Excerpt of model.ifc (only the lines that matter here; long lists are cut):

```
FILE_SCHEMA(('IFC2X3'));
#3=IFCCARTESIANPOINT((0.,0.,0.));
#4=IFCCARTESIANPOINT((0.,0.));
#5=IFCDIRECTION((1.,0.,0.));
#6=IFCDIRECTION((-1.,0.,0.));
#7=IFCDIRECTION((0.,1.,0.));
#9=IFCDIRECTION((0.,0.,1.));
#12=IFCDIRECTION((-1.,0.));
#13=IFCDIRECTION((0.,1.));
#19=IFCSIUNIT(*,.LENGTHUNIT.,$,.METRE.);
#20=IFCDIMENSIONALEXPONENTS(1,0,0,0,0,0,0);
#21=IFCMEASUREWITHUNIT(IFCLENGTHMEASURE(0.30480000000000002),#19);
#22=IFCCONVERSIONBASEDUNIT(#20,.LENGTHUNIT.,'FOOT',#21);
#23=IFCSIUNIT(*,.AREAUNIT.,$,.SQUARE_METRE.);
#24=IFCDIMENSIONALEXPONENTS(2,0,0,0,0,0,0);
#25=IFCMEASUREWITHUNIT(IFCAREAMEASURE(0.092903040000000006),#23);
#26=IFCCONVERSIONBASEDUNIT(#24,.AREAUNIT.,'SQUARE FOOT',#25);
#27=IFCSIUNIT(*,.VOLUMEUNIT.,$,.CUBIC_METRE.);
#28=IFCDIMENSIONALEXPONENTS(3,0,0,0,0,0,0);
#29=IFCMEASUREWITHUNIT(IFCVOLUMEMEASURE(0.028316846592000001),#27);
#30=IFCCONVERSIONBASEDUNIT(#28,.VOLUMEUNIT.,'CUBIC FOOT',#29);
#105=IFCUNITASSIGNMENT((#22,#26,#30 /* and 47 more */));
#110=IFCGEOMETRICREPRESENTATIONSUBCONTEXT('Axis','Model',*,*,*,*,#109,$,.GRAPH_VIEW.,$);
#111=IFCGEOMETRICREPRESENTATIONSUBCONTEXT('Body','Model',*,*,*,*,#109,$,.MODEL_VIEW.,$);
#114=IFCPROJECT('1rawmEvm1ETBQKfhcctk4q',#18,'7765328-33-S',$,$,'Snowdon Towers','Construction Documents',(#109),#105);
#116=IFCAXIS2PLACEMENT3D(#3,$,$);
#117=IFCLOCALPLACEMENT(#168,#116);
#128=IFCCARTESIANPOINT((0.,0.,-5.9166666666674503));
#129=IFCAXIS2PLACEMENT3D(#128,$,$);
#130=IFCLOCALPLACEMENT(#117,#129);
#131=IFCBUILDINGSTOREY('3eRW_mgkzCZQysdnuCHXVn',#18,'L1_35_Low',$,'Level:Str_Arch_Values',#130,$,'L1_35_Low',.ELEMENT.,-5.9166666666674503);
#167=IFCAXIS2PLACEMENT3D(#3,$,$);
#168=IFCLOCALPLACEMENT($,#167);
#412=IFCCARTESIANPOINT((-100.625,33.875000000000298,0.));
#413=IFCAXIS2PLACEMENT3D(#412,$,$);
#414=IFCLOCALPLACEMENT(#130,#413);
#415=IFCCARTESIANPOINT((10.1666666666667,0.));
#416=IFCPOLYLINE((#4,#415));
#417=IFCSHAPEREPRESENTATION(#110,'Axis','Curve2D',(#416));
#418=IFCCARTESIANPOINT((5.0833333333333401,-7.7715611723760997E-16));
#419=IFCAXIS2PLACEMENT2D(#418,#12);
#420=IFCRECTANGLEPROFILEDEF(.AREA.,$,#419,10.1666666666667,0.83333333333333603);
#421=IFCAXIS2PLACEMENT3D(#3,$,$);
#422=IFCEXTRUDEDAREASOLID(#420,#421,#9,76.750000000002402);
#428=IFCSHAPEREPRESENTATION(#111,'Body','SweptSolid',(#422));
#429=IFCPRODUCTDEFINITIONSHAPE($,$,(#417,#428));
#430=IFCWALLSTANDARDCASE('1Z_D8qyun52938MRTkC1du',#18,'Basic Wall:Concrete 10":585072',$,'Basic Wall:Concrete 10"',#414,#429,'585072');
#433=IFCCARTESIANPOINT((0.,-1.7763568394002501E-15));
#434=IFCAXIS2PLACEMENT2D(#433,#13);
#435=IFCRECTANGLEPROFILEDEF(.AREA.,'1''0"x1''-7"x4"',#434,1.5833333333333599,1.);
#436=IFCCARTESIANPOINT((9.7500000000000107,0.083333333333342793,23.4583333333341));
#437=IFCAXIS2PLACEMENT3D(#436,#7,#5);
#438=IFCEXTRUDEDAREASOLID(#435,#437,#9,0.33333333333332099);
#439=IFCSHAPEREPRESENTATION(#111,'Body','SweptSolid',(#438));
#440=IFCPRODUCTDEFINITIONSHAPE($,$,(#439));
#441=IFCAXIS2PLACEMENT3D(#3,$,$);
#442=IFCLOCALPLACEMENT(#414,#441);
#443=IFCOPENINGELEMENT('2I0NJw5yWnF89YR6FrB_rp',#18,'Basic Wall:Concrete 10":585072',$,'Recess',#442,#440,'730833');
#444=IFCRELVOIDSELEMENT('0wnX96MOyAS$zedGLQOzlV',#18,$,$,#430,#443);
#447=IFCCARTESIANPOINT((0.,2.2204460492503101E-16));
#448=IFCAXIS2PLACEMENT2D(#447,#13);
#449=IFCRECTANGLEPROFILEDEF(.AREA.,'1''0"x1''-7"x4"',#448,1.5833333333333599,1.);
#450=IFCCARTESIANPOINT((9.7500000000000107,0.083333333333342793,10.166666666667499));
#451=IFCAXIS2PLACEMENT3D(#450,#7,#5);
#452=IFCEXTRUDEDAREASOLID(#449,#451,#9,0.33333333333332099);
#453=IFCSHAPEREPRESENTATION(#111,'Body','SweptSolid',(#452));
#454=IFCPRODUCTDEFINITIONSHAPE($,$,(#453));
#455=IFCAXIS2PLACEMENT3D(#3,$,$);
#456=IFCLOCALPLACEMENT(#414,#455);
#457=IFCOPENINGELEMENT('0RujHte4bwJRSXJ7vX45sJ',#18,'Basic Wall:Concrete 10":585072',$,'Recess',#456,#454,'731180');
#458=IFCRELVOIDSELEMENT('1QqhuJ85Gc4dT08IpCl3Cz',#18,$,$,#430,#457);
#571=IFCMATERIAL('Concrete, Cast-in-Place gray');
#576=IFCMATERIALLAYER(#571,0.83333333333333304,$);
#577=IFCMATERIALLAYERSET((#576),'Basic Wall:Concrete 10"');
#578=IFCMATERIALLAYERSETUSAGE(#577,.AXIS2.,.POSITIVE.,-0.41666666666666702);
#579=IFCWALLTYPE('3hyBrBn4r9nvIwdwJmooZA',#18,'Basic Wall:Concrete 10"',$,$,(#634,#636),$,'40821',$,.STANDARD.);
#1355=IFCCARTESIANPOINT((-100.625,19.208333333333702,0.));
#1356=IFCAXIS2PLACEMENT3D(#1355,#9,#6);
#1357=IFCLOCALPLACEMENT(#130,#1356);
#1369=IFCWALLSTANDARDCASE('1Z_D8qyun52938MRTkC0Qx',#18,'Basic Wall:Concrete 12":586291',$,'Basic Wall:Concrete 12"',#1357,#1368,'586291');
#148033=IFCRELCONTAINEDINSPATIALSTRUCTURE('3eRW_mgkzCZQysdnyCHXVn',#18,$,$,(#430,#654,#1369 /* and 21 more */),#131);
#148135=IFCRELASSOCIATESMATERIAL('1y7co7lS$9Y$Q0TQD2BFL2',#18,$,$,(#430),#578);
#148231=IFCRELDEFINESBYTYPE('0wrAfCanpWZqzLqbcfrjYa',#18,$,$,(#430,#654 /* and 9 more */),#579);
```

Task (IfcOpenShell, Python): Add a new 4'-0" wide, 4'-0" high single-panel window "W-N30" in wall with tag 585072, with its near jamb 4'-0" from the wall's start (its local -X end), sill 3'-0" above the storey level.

```python
import numpy as np
import ifcopenshell
import ifcopenshell.api.feature
import ifcopenshell.api.geometry
import ifcopenshell.api.root
import ifcopenshell.api.spatial
import ifcopenshell.api.type
import ifcopenshell.geom
import ifcopenshell.util.element
import ifcopenshell.util.placement
import ifcopenshell.util.representation
import ifcopenshell.util.shape
import ifcopenshell.util.unit

model = ifcopenshell.open("model.ifc")
unit_scale = ifcopenshell.util.unit.calculate_unit_scale(model)
settings = ifcopenshell.geom.settings()


def volume(element):
    """Net volume in cubic metres, openings subtracted."""
    shape = ifcopenshell.geom.create_shape(settings, element)
    return ifcopenshell.util.shape.get_volume(shape.geometry)


wall = model.by_guid("1Z_D8qyun52938MRTkC1du")
storey = ifcopenshell.util.element.get_container(wall, ifc_class="IfcBuildingStorey")
context = ifcopenshell.util.representation.get_context(model, "Model", "Body", "MODEL_VIEW")
before = volume(wall)

width, height, from_end, sill = 1.2192, 1.2192, 1.2192, 0.9144  # metres

# The wall runs along its own X axis, and the end named is its -X end.
wall_shape = ifcopenshell.geom.create_shape(settings, wall)
x, y, z = ifcopenshell.util.shape.get_vertices(wall_shape.geometry).T
start = x.min() + from_end
face, thickness = float(y.min()), float(y.max() - y.min())
wall_matrix = ifcopenshell.util.placement.get_local_placement(wall.ObjectPlacement)
level = ifcopenshell.util.placement.get_local_placement(storey.ObjectPlacement)[2, 3]


def in_wall(x, y):
    """Placement at x, y metres in the wall's axes, at sill height."""
    matrix = wall_matrix.copy()
    matrix[:, 3] = wall_matrix @ np.array([x / unit_scale, y / unit_scale, 0.0, 1.0])
    matrix[2, 3] = level + sill / unit_scale
    return matrix


# Opening: a box that overshoots both wall faces by 50 mm.
opening = ifcopenshell.api.root.create_entity(model, ifc_class="IfcOpeningElement")
box = ifcopenshell.api.geometry.add_wall_representation(
    model, context=context, length=width, height=height, thickness=thickness + 0.1
)
ifcopenshell.api.geometry.assign_representation(model, product=opening, representation=box)
ifcopenshell.api.geometry.edit_object_placement(model, product=opening, matrix=in_wall(start, face - 0.05), is_si=False)
ifcopenshell.api.feature.add_feature(model, feature=opening, element=wall)

window = ifcopenshell.api.root.create_entity(model, ifc_class="IfcWindow", name="W-N30")
window.OverallWidth, window.OverallHeight = width / unit_scale, height / unit_scale
body = ifcopenshell.api.geometry.add_window_representation(
    model,
    context=context,
    overall_width=window.OverallWidth,
    overall_height=window.OverallHeight,
    partition_type="SINGLE_PANEL",
)
ifcopenshell.api.geometry.assign_representation(model, product=window, representation=body)
ifcopenshell.api.spatial.assign_container(model, products=[window], relating_structure=storey)
fills = ifcopenshell.api.feature.add_filling(model, opening=opening, element=window)
fills.OwnerHistory = window.OwnerHistory  # required in IFC2X3

# IFC2X3 keeps the operation on the window style.
style = ifcopenshell.api.root.create_entity(model, ifc_class="IfcWindowStyle", name="W-N30")
style.OperationType, style.ConstructionType = "SINGLE_PANEL", "NOTDEFINED"
style.ParameterTakesPrecedence = style.Sizeable = False
ifcopenshell.api.type.assign_type(model, related_objects=[window], relating_type=style)

# Centre the window in the wall's thickness.
ifcopenshell.api.geometry.edit_object_placement(model, product=window, matrix=in_wall(start, face), is_si=False)
window_shape = ifcopenshell.geom.create_shape(settings, window)
depth = ifcopenshell.util.shape.get_vertices(window_shape.geometry)[:, 1]
offset = face + thickness / 2 - (depth.min() + depth.max()) / 2
ifcopenshell.api.geometry.edit_object_placement(model, product=window, matrix=in_wall(start, offset), is_si=False)

after = volume(wall)

print(f"wall volume {before:.3f} -> {after:.3f} m3")

model.write("model_rev.ifc")
```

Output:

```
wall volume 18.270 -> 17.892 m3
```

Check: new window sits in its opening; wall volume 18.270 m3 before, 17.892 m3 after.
